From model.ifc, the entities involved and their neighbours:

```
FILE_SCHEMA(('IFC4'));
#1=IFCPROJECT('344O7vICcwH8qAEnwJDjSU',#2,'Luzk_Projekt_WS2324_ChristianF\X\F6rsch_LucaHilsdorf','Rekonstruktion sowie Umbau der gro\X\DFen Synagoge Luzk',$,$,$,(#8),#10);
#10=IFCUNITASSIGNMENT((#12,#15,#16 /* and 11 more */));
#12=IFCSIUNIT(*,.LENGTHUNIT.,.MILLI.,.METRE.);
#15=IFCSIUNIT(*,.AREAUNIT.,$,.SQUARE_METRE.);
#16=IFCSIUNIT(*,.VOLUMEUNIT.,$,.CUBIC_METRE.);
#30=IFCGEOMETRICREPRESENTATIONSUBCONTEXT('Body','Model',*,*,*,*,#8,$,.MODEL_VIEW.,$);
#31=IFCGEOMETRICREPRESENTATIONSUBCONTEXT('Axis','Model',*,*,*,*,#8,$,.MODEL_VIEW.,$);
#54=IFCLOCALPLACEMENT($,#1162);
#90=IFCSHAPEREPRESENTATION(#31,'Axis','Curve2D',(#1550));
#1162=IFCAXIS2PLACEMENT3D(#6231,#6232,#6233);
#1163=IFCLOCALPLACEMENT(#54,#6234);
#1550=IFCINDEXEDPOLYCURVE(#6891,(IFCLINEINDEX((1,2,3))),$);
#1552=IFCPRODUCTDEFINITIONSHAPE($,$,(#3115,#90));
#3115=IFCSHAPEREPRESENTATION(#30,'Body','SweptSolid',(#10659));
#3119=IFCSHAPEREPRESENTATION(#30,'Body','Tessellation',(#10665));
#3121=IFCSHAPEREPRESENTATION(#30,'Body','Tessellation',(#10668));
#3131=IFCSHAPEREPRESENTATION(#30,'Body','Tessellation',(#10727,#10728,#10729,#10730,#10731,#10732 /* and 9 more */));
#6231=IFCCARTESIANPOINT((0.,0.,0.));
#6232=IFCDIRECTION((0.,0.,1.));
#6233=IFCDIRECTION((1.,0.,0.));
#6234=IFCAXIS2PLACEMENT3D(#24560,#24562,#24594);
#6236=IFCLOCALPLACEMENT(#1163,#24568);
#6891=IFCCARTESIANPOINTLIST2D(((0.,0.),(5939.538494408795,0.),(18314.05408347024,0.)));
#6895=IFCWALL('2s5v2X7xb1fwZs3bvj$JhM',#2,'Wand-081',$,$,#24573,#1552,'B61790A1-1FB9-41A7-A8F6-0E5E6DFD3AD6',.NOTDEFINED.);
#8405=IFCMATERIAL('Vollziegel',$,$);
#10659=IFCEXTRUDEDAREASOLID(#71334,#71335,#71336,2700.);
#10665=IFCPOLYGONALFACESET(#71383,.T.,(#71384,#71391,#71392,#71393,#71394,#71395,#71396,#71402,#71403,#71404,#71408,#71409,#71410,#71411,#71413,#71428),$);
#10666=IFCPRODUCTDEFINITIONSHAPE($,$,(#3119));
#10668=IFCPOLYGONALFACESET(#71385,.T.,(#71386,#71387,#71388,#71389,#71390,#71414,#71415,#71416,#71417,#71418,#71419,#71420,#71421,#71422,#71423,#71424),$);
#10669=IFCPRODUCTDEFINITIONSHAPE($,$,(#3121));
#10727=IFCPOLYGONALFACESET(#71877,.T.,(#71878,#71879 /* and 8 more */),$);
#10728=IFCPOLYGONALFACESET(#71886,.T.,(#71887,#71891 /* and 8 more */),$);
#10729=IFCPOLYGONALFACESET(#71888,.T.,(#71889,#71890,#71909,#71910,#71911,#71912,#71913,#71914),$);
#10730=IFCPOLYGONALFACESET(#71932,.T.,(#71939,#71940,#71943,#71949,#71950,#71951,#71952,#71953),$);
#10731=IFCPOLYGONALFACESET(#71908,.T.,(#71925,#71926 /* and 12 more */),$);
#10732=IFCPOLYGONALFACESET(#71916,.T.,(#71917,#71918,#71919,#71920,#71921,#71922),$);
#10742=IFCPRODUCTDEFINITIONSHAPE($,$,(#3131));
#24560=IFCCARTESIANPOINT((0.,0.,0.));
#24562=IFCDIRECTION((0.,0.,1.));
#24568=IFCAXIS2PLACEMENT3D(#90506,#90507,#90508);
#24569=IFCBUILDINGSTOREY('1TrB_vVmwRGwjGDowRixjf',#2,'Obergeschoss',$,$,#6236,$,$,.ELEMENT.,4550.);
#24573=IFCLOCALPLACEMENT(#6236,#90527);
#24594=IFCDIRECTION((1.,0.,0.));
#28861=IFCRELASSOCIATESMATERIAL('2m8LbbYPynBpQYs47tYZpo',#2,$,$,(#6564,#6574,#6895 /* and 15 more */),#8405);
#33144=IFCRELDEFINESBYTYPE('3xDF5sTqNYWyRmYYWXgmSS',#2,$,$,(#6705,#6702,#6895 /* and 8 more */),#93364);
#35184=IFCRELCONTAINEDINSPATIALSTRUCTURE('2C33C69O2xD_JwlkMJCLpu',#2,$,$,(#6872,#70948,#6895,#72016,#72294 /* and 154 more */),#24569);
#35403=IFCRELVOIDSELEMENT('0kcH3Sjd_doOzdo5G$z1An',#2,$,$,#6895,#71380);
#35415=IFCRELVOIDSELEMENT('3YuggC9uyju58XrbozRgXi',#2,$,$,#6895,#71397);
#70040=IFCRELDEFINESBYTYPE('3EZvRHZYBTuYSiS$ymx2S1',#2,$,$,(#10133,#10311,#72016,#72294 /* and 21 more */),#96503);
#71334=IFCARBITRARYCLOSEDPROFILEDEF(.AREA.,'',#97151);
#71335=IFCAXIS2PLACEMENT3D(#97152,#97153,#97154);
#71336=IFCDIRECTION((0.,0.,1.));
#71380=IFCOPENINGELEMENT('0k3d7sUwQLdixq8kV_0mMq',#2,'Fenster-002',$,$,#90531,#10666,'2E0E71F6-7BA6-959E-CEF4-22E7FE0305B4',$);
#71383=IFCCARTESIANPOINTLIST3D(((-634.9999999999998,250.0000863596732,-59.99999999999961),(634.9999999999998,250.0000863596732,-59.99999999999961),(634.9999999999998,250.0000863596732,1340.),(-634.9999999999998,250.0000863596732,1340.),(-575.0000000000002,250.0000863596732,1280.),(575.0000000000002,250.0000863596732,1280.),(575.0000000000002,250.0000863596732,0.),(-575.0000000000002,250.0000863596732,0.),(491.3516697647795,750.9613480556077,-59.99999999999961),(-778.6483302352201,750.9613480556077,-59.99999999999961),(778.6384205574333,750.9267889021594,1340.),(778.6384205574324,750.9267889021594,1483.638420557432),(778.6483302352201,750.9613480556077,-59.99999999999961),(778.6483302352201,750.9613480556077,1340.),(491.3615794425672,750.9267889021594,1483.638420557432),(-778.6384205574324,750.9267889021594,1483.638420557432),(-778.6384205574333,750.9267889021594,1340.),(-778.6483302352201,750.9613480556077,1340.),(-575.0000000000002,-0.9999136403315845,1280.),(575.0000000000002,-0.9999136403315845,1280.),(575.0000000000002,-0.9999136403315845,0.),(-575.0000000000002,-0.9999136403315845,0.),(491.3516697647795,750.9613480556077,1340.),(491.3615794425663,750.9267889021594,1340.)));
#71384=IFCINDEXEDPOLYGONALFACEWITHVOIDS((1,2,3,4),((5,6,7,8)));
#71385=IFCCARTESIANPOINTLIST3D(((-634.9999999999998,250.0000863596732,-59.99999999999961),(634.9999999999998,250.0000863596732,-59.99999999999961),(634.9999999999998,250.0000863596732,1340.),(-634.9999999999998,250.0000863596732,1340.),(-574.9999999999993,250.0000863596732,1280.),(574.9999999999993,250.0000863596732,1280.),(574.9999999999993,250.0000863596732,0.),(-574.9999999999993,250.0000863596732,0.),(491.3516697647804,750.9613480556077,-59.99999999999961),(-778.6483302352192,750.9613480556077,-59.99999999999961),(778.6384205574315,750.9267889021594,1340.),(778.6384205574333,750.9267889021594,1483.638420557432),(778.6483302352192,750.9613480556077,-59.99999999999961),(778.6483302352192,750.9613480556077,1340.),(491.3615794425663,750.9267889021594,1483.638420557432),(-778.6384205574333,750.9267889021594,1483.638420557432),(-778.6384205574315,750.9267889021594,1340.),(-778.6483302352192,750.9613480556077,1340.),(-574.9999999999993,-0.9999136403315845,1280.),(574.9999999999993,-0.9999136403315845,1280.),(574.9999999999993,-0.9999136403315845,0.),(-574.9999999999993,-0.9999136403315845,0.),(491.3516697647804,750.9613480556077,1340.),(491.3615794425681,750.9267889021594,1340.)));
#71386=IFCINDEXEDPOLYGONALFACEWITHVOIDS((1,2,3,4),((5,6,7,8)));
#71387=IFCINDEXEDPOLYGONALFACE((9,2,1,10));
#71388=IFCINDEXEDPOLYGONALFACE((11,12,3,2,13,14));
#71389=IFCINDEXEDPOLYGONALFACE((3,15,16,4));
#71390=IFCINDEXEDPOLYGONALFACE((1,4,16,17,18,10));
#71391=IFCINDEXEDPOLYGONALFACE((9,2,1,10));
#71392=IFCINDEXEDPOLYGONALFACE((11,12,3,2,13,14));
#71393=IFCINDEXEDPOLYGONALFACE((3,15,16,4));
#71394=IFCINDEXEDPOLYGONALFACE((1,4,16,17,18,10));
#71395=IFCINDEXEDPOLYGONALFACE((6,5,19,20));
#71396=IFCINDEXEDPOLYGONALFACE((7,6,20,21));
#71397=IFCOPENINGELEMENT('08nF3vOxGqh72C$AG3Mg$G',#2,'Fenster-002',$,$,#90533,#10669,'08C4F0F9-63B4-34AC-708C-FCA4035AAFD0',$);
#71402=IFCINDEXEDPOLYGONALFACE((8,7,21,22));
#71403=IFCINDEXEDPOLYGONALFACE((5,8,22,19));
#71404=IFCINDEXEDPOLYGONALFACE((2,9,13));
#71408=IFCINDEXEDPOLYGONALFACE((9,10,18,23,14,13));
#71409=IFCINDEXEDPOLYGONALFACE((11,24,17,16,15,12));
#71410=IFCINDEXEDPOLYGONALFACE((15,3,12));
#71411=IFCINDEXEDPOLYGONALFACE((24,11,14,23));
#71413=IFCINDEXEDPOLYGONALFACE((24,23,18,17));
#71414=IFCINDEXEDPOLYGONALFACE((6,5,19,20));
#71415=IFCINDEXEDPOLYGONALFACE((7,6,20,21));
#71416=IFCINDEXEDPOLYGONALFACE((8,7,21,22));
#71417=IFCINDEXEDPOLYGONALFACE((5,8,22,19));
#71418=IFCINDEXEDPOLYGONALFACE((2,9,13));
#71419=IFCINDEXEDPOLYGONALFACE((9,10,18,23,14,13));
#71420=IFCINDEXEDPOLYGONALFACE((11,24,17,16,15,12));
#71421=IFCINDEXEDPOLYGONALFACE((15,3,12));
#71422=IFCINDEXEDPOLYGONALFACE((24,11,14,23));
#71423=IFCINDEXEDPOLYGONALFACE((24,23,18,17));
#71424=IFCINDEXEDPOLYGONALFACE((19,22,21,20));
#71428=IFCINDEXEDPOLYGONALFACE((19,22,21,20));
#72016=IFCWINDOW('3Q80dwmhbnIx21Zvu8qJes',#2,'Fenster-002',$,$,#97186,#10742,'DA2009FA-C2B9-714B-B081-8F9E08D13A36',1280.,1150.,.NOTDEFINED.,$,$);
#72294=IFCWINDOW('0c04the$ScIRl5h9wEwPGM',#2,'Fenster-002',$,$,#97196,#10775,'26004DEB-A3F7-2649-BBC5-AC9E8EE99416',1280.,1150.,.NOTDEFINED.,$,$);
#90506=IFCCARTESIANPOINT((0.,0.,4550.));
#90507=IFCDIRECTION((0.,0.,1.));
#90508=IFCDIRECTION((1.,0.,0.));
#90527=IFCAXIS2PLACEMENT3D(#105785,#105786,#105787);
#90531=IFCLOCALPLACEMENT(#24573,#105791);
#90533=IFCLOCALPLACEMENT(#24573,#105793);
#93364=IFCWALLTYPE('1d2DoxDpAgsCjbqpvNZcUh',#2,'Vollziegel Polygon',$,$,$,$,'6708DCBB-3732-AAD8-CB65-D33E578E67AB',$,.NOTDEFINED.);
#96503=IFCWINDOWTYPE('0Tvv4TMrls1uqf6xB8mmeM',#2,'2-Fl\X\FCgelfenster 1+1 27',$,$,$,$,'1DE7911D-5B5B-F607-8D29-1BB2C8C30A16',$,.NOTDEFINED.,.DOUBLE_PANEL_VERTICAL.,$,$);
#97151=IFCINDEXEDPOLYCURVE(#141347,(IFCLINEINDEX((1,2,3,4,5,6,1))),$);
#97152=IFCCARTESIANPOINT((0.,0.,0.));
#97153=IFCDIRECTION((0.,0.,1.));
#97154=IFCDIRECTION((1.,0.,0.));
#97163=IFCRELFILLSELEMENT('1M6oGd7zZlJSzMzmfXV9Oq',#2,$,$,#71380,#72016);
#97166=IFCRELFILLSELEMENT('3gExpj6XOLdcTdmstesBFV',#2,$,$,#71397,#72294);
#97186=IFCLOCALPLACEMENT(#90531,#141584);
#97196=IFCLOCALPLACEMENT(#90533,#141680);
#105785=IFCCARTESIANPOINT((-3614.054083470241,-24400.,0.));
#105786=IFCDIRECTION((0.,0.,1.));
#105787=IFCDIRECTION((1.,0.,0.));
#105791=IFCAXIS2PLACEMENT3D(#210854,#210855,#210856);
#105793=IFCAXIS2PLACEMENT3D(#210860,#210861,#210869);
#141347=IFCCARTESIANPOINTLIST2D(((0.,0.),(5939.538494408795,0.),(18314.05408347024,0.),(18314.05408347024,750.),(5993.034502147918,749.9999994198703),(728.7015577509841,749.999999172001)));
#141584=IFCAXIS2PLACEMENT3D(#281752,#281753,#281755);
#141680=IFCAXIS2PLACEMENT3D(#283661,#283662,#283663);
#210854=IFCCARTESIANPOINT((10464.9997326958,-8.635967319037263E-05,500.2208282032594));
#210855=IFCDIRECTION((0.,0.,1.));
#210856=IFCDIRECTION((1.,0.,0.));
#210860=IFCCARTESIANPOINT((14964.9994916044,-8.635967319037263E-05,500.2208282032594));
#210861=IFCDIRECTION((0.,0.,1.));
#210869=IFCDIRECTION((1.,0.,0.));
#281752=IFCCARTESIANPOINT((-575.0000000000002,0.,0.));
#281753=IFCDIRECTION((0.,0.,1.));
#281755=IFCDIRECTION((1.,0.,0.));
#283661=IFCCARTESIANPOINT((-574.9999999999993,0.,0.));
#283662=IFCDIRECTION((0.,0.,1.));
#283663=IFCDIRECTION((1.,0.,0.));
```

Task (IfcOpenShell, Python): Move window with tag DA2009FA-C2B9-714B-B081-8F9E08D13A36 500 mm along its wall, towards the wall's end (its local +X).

```python
import ifcopenshell
import ifcopenshell.api.geometry
import ifcopenshell.util.placement
import ifcopenshell.util.unit

model = ifcopenshell.open("model.ifc")
unit_scale = ifcopenshell.util.unit.calculate_unit_scale(model)

window = model.by_guid("3Q80dwmhbnIx21Zvu8qJes")
opening = window.FillsVoids[0].RelatingOpeningElement
wall = opening.VoidsElements[0].RelatingBuildingElement

wall_matrix = ifcopenshell.util.placement.get_local_placement(wall.ObjectPlacement)
shift = wall_matrix[:3, 0] * 0.5 / unit_scale
before = ifcopenshell.util.placement.get_local_placement(window.ObjectPlacement)[:3, 3].copy()

# The window is placed relative to its opening, so it follows when the opening moves.
matrix = ifcopenshell.util.placement.get_local_placement(opening.ObjectPlacement)
matrix[:3, 3] += shift
ifcopenshell.api.geometry.edit_object_placement(
    model, product=opening, matrix=matrix, is_si=False, should_transform_children=True
)

after = ifcopenshell.util.placement.get_local_placement(window.ObjectPlacement)[:3, 3]
print("window moved by", (after - before).round(3) + 0.0)

model.write("model_updated.ifc")
```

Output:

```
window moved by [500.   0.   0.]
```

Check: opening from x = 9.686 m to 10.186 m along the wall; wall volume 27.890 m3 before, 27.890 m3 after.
